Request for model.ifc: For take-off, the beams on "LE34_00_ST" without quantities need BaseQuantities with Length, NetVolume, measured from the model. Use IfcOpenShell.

First a look at what the model holds.

```python
import ifcopenshell
import ifcopenshell.util.element
import ifcopenshell.util.unit

model = ifcopenshell.open("model.ifc")
print(model.schema)
for unit_type in ("LENGTHUNIT", "AREAUNIT", "VOLUMEUNIT"):
    print(unit_type, ifcopenshell.util.unit.calculate_unit_scale(model, unit_type))
storey = next(s for s in model.by_type("IfcBuildingStorey") if s.Name == "LE34_00_ST")
beams = [e for e in ifcopenshell.util.element.get_decomposition(storey) if e.is_a("IfcBeam")]
for e in sorted(beams, key=lambda e: e.id()):
    print(e.id(), e.is_a(), e.Name, list(ifcopenshell.util.element.get_psets(e, qtos_only=True)), sep=" | ")
```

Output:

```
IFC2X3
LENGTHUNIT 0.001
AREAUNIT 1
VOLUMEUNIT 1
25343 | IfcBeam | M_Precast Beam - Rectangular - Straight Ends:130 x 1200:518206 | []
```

```python
import ifcopenshell
import ifcopenshell.api.pset
import ifcopenshell.geom
import ifcopenshell.util.element
import ifcopenshell.util.shape
import ifcopenshell.util.unit

model = ifcopenshell.open("model.ifc")
unit_scale = ifcopenshell.util.unit.calculate_unit_scale(model)
volume_scale = ifcopenshell.util.unit.calculate_unit_scale(model, "VOLUMEUNIT")
settings = ifcopenshell.geom.settings()

storey = next(s for s in model.by_type("IfcBuildingStorey") if s.Name == "LE34_00_ST")
beams = [e for e in ifcopenshell.util.element.get_decomposition(storey) if e.is_a("IfcBeam")]

for e in sorted(beams, key=lambda e: e.id()):
    if ifcopenshell.util.element.get_psets(e, qtos_only=True, should_inherit=False):
        continue
    # Geometry comes back in metres, in the element's own axes.
    shape = ifcopenshell.geom.create_shape(settings, e)
    values = {
        "Length": ifcopenshell.util.shape.get_max_xyz(shape.geometry) / unit_scale,
        "NetVolume": ifcopenshell.util.shape.get_volume(shape.geometry) / volume_scale,
    }
    qto = ifcopenshell.api.pset.add_qto(model, product=e, name="BaseQuantities")
    ifcopenshell.api.pset.edit_qto(model, qto=qto, properties=values)
    print(e.id(), {k: round(v, 3) for k, v in values.items()})

model.write("model_edited.ifc")
```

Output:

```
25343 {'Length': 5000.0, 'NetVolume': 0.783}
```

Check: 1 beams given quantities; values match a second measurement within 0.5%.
